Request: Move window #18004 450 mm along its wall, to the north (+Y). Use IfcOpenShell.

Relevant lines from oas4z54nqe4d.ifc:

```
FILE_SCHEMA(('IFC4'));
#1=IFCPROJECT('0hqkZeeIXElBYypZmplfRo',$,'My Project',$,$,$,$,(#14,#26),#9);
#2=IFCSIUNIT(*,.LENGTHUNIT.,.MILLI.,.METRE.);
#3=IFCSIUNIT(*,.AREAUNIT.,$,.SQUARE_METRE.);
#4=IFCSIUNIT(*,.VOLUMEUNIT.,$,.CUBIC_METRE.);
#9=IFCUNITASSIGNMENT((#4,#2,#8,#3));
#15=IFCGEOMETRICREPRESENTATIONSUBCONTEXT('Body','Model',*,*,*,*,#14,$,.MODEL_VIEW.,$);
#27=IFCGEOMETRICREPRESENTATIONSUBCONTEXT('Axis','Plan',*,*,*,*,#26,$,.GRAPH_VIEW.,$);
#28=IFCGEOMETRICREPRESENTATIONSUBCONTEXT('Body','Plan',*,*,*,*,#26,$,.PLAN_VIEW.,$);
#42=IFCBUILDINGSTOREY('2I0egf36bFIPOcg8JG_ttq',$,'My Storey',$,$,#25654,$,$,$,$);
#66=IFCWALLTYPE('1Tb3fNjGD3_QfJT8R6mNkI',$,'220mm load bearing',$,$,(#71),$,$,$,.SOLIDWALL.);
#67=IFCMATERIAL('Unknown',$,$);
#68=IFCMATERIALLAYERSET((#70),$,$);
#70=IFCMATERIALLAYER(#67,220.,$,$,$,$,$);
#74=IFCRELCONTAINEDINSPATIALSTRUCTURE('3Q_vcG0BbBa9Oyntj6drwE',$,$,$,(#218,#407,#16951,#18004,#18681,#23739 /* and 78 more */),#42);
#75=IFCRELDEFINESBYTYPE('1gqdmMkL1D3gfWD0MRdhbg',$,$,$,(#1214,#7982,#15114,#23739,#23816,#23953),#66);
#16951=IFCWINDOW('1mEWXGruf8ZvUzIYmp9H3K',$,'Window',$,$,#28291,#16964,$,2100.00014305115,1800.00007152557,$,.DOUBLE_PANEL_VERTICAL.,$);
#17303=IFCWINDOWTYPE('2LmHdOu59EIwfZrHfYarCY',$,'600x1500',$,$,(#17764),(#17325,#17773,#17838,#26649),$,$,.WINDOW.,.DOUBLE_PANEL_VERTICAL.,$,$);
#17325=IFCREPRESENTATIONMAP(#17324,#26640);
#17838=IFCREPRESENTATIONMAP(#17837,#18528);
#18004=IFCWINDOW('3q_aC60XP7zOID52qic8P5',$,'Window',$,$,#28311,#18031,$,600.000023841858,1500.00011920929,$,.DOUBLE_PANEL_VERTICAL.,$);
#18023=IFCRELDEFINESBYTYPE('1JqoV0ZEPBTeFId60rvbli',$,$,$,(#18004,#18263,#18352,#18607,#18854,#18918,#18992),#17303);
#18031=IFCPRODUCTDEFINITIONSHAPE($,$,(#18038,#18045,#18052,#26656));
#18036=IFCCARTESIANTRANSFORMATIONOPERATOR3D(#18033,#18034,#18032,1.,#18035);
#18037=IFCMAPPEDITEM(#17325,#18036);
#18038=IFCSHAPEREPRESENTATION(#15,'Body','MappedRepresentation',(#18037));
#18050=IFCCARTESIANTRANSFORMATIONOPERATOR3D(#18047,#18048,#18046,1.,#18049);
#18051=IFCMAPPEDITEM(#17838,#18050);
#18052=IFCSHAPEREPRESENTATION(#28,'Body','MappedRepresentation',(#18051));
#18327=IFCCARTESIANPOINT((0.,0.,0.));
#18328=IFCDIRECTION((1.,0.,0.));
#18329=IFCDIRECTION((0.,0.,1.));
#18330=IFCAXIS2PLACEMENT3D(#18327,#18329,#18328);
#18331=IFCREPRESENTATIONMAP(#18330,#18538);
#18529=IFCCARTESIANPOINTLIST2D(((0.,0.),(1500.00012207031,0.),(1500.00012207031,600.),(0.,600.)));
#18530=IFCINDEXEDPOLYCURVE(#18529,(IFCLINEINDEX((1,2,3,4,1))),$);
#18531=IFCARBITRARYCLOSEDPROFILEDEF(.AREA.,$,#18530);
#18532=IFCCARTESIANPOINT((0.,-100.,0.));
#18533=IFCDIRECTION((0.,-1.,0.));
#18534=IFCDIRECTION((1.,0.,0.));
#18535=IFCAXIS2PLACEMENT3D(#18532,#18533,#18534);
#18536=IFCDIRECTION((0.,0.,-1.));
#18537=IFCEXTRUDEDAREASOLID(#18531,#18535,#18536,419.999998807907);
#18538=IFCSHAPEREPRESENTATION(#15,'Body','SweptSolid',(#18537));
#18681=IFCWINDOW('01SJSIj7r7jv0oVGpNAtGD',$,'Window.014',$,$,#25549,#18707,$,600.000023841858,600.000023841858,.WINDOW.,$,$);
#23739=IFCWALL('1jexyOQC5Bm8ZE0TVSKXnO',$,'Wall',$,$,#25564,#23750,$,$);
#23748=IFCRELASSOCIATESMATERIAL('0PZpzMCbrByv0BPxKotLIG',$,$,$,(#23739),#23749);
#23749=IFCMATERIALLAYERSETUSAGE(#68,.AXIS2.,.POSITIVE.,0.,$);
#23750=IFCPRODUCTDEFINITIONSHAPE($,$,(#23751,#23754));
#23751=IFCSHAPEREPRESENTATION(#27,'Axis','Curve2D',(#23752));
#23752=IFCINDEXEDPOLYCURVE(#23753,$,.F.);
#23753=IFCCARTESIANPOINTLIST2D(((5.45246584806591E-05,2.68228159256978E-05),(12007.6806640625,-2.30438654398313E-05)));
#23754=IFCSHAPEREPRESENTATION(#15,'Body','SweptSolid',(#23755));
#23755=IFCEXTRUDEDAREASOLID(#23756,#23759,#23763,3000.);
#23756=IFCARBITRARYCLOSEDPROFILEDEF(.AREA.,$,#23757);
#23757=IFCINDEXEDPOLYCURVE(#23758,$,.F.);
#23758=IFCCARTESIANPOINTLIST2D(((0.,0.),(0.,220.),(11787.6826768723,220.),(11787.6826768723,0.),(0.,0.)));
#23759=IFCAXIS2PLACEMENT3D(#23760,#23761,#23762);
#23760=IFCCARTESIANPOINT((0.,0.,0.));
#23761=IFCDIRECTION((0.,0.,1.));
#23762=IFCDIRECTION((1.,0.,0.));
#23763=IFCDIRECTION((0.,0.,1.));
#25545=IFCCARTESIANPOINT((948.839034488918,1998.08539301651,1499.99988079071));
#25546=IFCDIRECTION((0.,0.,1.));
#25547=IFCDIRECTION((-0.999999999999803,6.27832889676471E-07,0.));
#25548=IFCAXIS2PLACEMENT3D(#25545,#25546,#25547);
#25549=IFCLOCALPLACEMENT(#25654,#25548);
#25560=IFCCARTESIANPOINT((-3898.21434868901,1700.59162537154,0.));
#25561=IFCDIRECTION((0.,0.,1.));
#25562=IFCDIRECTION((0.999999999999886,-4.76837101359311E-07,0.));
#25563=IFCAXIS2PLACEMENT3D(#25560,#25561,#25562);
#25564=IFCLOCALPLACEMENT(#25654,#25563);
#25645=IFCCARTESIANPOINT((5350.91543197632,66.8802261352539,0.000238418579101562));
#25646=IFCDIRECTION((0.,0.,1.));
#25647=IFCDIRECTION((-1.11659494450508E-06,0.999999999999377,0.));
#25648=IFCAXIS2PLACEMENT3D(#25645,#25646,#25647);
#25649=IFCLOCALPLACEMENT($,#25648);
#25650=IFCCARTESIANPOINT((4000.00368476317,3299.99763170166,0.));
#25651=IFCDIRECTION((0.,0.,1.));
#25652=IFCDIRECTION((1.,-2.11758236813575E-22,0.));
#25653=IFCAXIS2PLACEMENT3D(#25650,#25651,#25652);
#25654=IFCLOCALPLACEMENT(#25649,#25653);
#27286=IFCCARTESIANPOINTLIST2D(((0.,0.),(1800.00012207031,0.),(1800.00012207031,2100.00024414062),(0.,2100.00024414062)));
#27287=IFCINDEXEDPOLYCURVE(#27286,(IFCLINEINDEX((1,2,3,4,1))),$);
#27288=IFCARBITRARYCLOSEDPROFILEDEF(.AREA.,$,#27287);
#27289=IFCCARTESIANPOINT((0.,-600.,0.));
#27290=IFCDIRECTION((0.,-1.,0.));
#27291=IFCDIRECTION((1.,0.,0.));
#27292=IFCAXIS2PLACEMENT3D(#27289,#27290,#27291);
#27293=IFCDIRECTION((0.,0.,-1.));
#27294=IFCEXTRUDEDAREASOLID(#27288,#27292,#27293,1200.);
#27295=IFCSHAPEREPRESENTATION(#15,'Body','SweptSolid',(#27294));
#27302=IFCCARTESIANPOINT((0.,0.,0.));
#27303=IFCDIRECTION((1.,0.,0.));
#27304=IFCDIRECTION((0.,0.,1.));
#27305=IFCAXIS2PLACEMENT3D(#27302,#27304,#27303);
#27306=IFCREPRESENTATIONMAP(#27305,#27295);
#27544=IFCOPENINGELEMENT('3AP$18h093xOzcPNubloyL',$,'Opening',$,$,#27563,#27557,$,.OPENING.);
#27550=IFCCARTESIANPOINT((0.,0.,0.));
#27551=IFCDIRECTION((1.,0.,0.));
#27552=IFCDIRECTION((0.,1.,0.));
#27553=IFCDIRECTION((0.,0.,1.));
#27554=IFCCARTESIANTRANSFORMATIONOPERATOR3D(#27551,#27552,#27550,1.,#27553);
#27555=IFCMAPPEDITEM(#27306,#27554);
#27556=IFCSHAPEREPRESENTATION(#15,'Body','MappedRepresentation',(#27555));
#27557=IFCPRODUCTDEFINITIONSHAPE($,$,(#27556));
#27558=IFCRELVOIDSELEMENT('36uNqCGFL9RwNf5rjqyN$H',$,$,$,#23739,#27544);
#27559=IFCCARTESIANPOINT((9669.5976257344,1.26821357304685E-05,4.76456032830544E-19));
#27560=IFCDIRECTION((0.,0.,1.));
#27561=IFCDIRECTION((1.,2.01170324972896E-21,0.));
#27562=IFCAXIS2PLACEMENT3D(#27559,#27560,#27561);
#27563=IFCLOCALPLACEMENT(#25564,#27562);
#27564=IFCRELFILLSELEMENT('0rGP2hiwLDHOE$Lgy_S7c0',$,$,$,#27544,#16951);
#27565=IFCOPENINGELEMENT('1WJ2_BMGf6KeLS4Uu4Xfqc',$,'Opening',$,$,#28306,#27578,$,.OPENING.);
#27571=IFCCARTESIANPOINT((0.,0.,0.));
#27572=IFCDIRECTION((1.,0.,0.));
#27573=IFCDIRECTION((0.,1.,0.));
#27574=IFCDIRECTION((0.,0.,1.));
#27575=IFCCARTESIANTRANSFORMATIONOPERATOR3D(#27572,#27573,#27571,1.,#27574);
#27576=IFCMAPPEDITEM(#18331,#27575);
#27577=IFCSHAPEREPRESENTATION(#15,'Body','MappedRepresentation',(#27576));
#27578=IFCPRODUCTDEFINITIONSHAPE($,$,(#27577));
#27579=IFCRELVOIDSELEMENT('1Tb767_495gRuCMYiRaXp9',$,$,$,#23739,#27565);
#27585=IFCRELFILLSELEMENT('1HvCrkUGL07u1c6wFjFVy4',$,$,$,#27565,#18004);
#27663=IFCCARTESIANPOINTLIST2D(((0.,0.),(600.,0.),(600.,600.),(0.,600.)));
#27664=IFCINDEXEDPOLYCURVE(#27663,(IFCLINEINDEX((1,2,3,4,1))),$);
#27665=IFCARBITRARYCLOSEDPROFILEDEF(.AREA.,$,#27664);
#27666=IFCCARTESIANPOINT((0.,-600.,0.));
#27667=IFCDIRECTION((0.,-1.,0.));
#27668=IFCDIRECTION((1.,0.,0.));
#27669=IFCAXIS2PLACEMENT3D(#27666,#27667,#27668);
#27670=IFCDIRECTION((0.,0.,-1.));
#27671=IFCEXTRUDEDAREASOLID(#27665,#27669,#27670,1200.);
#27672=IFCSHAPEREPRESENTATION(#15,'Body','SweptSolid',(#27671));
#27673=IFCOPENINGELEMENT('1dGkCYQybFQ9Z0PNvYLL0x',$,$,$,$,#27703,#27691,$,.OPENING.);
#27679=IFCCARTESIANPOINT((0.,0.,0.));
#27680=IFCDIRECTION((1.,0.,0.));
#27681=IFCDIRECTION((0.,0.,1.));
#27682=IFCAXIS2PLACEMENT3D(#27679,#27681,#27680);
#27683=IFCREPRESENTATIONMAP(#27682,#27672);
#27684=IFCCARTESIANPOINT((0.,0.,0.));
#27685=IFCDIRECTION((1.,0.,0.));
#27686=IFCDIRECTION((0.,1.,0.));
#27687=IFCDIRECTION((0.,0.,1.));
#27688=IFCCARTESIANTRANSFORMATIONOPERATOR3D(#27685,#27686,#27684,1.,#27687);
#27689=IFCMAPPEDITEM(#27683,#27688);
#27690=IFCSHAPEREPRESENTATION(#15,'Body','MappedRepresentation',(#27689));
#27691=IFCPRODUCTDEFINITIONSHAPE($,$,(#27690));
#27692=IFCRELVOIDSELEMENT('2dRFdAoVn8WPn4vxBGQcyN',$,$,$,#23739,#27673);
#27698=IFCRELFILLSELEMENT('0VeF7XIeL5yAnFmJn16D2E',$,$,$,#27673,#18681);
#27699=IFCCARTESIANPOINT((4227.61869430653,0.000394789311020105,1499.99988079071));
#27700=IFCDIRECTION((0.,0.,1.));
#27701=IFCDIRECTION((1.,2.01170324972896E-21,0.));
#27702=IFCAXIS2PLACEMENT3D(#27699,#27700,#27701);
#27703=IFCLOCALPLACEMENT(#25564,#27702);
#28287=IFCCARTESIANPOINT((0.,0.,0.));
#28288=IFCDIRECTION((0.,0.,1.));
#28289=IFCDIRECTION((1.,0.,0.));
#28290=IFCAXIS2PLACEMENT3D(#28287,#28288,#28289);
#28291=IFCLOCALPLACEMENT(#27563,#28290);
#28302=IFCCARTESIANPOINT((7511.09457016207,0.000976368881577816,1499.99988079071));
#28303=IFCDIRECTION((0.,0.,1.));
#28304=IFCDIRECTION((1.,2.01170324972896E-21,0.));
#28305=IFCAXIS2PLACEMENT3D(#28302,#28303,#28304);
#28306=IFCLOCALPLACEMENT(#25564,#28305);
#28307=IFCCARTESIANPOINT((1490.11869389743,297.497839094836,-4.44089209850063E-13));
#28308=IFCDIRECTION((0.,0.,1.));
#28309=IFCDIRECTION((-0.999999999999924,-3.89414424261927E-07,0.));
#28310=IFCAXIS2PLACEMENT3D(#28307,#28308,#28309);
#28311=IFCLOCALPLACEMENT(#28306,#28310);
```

```python
import ifcopenshell
import ifcopenshell.api.geometry
import ifcopenshell.util.placement
import ifcopenshell.util.unit

model = ifcopenshell.open("oas4z54nqe4d.ifc")
unit_scale = ifcopenshell.util.unit.calculate_unit_scale(model)

window = model.by_guid("3q_aC60XP7zOID52qic8P5")
opening = window.FillsVoids[0].RelatingOpeningElement
wall = opening.VoidsElements[0].RelatingBuildingElement

wall_matrix = ifcopenshell.util.placement.get_local_placement(wall.ObjectPlacement)
shift = wall_matrix[:3, 0] * 0.45 / unit_scale
before = ifcopenshell.util.placement.get_local_placement(window.ObjectPlacement)[:3, 3].copy()

# The window is placed relative to its opening, so it follows when the opening moves.
matrix = ifcopenshell.util.placement.get_local_placement(opening.ObjectPlacement)
matrix[:3, 3] += shift
ifcopenshell.api.geometry.edit_object_placement(
    model, product=opening, matrix=matrix, is_si=False, should_transform_children=True
)

after = ifcopenshell.util.placement.get_local_placement(window.ObjectPlacement)[:3, 3]
print("window moved by", (after - before).round(3) + 0.0)

model.write("oas4z54nqe4d_updated.ifc")
```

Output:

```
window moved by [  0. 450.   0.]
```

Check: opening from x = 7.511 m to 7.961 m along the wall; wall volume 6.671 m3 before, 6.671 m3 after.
